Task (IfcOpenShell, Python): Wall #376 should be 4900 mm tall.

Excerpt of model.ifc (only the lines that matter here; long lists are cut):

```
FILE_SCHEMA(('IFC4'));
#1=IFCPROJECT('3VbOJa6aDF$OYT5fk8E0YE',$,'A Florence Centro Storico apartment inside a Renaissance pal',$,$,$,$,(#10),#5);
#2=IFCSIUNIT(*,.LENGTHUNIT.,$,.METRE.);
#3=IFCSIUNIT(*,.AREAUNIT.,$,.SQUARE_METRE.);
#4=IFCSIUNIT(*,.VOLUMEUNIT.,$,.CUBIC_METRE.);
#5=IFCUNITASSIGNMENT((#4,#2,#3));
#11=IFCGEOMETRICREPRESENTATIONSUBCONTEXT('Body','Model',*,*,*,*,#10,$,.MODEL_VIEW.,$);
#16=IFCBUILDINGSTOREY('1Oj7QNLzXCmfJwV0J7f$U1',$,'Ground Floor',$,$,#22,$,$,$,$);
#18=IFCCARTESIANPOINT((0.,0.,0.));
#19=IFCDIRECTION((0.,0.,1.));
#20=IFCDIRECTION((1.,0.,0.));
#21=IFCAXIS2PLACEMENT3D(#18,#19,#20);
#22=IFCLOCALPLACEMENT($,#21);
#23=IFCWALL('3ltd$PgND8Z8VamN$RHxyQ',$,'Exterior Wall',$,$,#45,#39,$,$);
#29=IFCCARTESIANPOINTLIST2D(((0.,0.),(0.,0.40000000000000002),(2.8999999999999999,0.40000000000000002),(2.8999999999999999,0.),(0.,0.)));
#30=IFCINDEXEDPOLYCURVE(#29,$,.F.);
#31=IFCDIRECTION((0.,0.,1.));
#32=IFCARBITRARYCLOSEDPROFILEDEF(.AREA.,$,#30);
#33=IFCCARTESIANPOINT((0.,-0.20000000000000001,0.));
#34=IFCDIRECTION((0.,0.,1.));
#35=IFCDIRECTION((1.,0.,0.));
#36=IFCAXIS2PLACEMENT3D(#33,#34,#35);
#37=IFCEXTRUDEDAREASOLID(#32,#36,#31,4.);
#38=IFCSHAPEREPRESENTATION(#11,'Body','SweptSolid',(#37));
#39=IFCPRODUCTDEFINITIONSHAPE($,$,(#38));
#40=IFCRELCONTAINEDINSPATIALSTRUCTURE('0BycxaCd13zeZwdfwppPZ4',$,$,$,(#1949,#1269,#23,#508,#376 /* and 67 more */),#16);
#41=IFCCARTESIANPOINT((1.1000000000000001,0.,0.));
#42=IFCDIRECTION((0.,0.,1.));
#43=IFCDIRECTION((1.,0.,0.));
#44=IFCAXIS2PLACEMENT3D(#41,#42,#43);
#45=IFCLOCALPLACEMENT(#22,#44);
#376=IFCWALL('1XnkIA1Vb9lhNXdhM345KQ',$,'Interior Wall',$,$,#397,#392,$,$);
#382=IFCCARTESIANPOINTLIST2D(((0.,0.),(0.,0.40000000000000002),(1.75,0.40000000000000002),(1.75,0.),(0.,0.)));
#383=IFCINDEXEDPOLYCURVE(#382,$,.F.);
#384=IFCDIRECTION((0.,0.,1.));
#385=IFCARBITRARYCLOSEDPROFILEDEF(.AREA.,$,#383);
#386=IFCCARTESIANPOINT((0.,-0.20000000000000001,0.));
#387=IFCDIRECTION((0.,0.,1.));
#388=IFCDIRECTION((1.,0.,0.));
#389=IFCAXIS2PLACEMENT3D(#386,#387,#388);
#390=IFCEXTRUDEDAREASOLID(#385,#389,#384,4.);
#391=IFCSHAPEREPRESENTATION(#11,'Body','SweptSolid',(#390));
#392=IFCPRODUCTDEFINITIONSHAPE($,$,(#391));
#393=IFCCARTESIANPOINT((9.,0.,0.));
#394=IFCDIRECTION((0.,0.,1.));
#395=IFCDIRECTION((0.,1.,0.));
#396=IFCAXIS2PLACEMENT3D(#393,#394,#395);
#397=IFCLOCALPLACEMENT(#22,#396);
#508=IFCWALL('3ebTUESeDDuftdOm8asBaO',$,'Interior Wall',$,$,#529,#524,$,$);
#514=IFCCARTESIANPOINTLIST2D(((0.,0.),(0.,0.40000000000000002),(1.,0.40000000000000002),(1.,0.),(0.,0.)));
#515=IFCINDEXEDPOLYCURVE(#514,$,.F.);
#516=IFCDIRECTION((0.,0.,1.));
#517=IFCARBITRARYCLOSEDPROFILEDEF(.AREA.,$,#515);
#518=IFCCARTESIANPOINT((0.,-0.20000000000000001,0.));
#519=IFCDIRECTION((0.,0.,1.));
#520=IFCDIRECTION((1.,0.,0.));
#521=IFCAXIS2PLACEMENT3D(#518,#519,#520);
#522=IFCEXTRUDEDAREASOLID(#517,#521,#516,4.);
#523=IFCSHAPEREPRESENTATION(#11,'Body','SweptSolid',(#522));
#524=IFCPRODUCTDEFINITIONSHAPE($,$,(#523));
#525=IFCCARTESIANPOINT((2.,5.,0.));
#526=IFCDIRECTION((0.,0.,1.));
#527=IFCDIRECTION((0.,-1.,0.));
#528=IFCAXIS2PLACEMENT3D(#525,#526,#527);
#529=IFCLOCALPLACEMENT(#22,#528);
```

```python
import ifcopenshell
import ifcopenshell.geom
import ifcopenshell.util.representation
import ifcopenshell.util.shape
import ifcopenshell.util.unit

model = ifcopenshell.open("model.ifc")
unit_scale = ifcopenshell.util.unit.calculate_unit_scale(model)
settings = ifcopenshell.geom.settings()


def volume(element):
    """Net volume in cubic metres, openings subtracted."""
    shape = ifcopenshell.geom.create_shape(settings, element)
    return ifcopenshell.util.shape.get_volume(shape.geometry)


wall = model.by_guid("1XnkIA1Vb9lhNXdhM345KQ")
before = volume(wall)

body = ifcopenshell.util.representation.get_representation(wall, "Model", "Body")
solid = body.Items[0]
old_height = solid.Depth
solid.Depth = 4.9 / unit_scale
after = volume(wall)

print(f"height {old_height:g} -> {solid.Depth:g}, volume {before:.3f} -> {after:.3f} m3")

model.write("model_v2.ifc")
```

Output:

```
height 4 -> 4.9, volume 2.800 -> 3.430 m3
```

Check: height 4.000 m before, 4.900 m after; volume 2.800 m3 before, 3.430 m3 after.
